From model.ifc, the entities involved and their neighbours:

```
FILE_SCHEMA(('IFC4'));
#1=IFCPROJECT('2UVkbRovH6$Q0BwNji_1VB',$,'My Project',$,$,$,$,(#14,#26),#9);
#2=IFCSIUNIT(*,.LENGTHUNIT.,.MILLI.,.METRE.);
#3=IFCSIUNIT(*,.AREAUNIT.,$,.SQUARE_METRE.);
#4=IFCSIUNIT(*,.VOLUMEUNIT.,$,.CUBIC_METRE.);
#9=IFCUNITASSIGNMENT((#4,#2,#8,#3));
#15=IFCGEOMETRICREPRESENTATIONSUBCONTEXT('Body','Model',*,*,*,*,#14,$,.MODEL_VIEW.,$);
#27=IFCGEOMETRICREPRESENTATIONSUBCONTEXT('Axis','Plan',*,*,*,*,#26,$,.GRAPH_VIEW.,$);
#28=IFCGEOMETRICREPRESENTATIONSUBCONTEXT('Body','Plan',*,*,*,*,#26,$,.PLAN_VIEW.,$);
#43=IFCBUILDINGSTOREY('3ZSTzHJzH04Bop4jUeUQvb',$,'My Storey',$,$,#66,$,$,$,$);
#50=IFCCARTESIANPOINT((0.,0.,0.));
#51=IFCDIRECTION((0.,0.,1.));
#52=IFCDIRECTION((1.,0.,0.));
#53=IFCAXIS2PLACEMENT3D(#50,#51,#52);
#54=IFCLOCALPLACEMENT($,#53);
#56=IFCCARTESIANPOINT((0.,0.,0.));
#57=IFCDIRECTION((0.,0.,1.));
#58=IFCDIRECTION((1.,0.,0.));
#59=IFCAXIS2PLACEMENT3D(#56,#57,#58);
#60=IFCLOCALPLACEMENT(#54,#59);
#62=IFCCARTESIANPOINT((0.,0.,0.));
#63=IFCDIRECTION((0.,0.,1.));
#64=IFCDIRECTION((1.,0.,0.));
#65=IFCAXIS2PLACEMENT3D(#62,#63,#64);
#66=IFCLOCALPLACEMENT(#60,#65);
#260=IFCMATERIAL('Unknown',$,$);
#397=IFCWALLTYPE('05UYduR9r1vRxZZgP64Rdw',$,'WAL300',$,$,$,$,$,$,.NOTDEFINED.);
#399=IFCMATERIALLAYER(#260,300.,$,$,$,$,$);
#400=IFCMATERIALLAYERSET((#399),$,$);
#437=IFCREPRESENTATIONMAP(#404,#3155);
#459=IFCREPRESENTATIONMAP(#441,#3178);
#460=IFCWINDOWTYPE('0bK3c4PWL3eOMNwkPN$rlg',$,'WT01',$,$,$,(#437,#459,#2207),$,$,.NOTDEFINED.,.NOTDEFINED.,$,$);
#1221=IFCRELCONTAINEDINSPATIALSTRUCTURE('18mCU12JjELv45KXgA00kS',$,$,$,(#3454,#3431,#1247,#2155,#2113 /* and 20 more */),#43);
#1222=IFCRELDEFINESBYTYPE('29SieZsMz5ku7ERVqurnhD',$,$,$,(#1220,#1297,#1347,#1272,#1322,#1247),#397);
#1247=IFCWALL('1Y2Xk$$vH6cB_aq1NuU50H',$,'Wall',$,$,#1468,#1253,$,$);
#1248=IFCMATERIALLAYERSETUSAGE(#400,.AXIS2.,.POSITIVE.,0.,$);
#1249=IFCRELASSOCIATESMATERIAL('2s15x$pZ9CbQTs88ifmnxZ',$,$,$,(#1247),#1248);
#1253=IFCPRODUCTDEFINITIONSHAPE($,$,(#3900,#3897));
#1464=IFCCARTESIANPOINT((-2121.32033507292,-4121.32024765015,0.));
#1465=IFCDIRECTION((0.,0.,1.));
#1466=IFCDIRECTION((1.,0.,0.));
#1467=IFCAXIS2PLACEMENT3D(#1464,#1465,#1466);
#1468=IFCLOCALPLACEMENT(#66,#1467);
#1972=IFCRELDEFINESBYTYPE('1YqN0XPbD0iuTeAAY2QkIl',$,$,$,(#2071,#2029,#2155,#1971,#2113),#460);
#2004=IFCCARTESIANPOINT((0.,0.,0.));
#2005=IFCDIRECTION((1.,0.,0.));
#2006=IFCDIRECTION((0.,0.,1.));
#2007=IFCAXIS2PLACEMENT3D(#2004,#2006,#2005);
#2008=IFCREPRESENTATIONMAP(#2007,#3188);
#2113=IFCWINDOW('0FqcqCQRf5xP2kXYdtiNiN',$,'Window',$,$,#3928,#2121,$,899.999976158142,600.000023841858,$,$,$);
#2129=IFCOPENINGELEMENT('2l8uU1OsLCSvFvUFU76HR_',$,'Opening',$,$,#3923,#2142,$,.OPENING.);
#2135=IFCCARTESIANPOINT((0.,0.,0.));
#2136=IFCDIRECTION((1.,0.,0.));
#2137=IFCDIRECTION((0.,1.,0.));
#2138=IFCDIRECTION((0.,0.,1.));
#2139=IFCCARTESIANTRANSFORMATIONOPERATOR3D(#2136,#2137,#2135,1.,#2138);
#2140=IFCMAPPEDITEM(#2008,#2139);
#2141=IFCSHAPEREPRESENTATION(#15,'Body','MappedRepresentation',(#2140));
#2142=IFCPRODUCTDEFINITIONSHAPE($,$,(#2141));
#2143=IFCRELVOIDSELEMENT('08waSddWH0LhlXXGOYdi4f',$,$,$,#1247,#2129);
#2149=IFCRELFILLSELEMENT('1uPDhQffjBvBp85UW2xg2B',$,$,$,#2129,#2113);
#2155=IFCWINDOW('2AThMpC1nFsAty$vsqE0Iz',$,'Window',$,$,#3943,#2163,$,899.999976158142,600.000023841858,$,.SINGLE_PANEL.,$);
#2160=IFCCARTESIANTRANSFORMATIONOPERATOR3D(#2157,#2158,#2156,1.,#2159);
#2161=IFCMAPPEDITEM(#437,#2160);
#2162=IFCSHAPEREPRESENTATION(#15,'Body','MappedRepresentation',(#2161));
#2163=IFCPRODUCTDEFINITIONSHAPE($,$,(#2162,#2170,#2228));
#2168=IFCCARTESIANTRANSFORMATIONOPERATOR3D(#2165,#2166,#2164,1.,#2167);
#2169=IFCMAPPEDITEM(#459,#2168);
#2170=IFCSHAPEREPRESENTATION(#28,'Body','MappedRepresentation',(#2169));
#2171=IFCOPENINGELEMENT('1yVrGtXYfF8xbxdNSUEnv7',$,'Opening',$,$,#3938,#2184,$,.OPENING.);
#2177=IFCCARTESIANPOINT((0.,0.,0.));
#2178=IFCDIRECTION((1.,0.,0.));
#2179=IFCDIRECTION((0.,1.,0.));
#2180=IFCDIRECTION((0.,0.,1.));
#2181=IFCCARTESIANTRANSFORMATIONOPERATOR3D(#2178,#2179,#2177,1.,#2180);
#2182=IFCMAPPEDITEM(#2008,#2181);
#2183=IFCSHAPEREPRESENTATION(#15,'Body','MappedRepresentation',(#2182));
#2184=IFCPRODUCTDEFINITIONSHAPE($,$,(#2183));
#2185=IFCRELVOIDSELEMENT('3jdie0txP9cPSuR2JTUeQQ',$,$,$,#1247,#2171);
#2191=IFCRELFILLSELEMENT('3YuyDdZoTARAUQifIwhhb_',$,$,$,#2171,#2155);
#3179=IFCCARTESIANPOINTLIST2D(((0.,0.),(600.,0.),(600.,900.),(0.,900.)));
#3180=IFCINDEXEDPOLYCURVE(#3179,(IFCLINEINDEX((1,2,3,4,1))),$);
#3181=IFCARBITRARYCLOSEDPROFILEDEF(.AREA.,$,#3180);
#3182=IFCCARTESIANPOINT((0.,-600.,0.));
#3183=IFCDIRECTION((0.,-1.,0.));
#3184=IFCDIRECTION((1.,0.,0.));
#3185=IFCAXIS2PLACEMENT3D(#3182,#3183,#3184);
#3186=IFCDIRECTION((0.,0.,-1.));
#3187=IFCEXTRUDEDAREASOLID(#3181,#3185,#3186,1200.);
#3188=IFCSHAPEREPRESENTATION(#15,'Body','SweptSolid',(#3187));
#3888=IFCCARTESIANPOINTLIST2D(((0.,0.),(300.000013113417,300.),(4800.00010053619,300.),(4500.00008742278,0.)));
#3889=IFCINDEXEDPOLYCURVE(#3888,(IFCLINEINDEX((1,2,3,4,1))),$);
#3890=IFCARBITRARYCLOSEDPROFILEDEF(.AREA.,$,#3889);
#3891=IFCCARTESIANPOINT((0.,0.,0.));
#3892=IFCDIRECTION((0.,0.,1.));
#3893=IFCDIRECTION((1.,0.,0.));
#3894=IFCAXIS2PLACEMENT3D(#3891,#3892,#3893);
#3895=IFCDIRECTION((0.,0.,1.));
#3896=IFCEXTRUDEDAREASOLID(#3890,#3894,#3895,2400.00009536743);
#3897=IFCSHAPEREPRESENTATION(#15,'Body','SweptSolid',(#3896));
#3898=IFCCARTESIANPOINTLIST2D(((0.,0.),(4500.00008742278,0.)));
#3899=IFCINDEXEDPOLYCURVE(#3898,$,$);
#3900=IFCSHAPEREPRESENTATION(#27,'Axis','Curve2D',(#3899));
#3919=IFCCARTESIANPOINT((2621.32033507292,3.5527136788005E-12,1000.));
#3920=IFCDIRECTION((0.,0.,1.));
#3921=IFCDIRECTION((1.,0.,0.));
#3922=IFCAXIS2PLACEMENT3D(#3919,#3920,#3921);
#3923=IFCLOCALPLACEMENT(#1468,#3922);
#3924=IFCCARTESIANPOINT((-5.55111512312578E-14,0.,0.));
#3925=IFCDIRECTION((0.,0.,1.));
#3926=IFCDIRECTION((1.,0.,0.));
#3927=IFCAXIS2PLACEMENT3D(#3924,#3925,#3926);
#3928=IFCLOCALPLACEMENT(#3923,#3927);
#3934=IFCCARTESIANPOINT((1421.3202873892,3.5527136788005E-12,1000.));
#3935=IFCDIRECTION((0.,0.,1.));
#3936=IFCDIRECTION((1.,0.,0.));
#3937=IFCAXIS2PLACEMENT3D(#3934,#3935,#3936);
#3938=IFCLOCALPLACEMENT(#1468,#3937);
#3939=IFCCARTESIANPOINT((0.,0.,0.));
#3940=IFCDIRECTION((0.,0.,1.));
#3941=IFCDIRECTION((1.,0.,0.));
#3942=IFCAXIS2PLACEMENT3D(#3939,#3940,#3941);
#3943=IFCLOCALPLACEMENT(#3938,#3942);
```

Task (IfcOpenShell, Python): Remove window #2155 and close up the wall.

```python
import ifcopenshell
import ifcopenshell.api.feature
import ifcopenshell.api.root
import ifcopenshell.geom
import ifcopenshell.util.shape

model = ifcopenshell.open("model.ifc")
settings = ifcopenshell.geom.settings()


def volume(element):
    """Net volume in cubic metres, openings subtracted."""
    shape = ifcopenshell.geom.create_shape(settings, element)
    return ifcopenshell.util.shape.get_volume(shape.geometry)


window = model.by_guid("2AThMpC1nFsAty$vsqE0Iz")
opening = window.FillsVoids[0].RelatingOpeningElement
wall = opening.VoidsElements[0].RelatingBuildingElement
before = volume(wall)

ifcopenshell.api.root.remove_product(model, product=window)
ifcopenshell.api.feature.remove_feature(model, feature=opening)

after = volume(wall)

print(f"wall volume {before:.3f} -> {after:.3f} m3")

model.write("model-out.ifc")
```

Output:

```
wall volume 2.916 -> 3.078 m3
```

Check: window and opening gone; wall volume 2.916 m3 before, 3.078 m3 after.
